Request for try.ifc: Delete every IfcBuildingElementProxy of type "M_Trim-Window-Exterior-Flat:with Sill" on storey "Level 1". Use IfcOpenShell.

First a look at what the model holds.

```python
import ifcopenshell
import ifcopenshell.util.element

model = ifcopenshell.open("try.ifc")
print(model.schema)
storey = next(s for s in model.by_type("IfcBuildingStorey") if s.Name == "Level 1")
proxies = [e for e in ifcopenshell.util.element.get_decomposition(storey) if e.is_a("IfcBuildingElementProxy")]
seen = {}
for e in proxies:
    element_type = ifcopenshell.util.element.get_type(e)
    name = element_type.Name if element_type not in (None, e) else None
    seen[name] = seen.get(name, 0) + 1
for name, count in sorted(seen.items(), key=str):
    print(count, "x", name)
```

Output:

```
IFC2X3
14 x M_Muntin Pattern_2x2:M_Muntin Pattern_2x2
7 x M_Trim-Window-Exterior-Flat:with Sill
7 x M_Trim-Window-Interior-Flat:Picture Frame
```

```python
import ifcopenshell
import ifcopenshell.api.root
import ifcopenshell.util.element

model = ifcopenshell.open("try.ifc")

storey = next(s for s in model.by_type("IfcBuildingStorey") if s.Name == "Level 1")
proxies = [e for e in ifcopenshell.util.element.get_decomposition(storey) if e.is_a("IfcBuildingElementProxy")]
targets = [e for e in proxies if (t := ifcopenshell.util.element.get_type(e)) not in (None, e) and t.Name == "M_Trim-Window-Exterior-Flat:with Sill"]

for e in targets:
    ifcopenshell.api.root.remove_product(model, product=e)
print(len(targets), "removed")

model.write("try_v2.ifc")
```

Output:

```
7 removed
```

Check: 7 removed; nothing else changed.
